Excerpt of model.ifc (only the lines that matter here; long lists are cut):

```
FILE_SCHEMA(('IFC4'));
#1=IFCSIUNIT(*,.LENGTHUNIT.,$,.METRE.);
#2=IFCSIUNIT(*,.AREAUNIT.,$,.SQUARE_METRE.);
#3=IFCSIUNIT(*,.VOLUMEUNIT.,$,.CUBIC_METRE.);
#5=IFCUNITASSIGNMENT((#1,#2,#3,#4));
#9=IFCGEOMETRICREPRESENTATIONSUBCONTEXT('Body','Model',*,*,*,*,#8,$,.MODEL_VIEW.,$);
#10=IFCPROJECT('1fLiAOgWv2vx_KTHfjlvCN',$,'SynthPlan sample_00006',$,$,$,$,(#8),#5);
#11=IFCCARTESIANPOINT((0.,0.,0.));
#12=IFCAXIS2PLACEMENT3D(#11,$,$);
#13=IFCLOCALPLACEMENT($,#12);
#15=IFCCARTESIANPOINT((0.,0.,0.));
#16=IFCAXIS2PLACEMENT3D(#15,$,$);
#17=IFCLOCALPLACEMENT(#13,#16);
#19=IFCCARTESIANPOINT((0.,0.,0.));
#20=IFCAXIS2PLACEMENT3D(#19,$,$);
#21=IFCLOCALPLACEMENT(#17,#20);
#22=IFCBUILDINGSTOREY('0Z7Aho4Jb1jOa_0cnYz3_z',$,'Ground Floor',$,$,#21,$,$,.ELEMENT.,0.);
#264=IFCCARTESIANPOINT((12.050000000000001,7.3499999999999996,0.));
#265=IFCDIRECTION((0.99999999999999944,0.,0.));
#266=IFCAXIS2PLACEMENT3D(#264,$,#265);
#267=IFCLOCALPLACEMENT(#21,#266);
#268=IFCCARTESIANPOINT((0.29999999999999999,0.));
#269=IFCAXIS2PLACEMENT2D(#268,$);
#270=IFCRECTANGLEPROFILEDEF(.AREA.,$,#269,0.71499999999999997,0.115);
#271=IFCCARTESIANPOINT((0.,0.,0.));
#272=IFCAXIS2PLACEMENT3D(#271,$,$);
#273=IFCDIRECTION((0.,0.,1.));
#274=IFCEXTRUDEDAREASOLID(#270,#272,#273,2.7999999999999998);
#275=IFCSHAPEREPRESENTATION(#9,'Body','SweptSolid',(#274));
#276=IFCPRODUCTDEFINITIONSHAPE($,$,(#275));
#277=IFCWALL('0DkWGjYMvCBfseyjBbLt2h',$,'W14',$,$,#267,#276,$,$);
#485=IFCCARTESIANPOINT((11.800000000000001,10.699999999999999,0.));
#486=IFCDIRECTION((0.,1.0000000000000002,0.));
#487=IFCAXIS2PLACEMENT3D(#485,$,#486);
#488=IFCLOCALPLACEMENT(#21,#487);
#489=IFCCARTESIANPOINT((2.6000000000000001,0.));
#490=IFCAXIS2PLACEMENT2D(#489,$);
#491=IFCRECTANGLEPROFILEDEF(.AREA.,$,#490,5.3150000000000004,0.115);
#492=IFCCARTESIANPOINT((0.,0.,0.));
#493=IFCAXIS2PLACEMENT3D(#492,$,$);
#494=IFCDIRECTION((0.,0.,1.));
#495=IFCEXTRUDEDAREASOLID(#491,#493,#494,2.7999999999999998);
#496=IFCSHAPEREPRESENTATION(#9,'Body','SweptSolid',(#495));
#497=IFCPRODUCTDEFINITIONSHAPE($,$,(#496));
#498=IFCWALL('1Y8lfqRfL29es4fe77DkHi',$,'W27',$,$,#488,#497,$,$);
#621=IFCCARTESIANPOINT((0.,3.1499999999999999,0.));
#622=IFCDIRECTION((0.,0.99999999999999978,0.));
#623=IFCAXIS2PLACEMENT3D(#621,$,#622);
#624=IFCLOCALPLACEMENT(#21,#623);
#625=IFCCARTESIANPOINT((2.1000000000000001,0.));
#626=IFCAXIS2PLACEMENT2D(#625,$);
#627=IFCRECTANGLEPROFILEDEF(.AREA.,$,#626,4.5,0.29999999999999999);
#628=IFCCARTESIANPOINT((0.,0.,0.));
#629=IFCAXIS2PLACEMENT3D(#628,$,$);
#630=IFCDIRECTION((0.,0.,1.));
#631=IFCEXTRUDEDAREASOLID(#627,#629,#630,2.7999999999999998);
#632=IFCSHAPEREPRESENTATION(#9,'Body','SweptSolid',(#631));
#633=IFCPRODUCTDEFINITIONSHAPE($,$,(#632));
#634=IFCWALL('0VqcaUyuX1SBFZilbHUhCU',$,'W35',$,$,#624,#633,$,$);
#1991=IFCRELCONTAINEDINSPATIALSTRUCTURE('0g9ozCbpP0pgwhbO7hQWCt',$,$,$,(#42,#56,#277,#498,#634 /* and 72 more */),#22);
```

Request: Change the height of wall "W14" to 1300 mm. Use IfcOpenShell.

```python
import ifcopenshell
import ifcopenshell.geom
import ifcopenshell.util.representation
import ifcopenshell.util.shape
import ifcopenshell.util.unit

model = ifcopenshell.open("model.ifc")
unit_scale = ifcopenshell.util.unit.calculate_unit_scale(model)
settings = ifcopenshell.geom.settings()


def volume(element):
    """Net volume in cubic metres, openings subtracted."""
    shape = ifcopenshell.geom.create_shape(settings, element)
    return ifcopenshell.util.shape.get_volume(shape.geometry)


wall = model.by_id(277)
before = volume(wall)

body = ifcopenshell.util.representation.get_representation(wall, "Model", "Body")
solid = body.Items[0]
old_height = solid.Depth
solid.Depth = 1.3 / unit_scale
after = volume(wall)

print(f"height {old_height:g} -> {solid.Depth:g}, volume {before:.3f} -> {after:.3f} m3")

model.write("model-out.ifc")
```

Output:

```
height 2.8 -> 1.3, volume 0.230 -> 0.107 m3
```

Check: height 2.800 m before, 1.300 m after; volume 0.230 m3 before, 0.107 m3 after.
